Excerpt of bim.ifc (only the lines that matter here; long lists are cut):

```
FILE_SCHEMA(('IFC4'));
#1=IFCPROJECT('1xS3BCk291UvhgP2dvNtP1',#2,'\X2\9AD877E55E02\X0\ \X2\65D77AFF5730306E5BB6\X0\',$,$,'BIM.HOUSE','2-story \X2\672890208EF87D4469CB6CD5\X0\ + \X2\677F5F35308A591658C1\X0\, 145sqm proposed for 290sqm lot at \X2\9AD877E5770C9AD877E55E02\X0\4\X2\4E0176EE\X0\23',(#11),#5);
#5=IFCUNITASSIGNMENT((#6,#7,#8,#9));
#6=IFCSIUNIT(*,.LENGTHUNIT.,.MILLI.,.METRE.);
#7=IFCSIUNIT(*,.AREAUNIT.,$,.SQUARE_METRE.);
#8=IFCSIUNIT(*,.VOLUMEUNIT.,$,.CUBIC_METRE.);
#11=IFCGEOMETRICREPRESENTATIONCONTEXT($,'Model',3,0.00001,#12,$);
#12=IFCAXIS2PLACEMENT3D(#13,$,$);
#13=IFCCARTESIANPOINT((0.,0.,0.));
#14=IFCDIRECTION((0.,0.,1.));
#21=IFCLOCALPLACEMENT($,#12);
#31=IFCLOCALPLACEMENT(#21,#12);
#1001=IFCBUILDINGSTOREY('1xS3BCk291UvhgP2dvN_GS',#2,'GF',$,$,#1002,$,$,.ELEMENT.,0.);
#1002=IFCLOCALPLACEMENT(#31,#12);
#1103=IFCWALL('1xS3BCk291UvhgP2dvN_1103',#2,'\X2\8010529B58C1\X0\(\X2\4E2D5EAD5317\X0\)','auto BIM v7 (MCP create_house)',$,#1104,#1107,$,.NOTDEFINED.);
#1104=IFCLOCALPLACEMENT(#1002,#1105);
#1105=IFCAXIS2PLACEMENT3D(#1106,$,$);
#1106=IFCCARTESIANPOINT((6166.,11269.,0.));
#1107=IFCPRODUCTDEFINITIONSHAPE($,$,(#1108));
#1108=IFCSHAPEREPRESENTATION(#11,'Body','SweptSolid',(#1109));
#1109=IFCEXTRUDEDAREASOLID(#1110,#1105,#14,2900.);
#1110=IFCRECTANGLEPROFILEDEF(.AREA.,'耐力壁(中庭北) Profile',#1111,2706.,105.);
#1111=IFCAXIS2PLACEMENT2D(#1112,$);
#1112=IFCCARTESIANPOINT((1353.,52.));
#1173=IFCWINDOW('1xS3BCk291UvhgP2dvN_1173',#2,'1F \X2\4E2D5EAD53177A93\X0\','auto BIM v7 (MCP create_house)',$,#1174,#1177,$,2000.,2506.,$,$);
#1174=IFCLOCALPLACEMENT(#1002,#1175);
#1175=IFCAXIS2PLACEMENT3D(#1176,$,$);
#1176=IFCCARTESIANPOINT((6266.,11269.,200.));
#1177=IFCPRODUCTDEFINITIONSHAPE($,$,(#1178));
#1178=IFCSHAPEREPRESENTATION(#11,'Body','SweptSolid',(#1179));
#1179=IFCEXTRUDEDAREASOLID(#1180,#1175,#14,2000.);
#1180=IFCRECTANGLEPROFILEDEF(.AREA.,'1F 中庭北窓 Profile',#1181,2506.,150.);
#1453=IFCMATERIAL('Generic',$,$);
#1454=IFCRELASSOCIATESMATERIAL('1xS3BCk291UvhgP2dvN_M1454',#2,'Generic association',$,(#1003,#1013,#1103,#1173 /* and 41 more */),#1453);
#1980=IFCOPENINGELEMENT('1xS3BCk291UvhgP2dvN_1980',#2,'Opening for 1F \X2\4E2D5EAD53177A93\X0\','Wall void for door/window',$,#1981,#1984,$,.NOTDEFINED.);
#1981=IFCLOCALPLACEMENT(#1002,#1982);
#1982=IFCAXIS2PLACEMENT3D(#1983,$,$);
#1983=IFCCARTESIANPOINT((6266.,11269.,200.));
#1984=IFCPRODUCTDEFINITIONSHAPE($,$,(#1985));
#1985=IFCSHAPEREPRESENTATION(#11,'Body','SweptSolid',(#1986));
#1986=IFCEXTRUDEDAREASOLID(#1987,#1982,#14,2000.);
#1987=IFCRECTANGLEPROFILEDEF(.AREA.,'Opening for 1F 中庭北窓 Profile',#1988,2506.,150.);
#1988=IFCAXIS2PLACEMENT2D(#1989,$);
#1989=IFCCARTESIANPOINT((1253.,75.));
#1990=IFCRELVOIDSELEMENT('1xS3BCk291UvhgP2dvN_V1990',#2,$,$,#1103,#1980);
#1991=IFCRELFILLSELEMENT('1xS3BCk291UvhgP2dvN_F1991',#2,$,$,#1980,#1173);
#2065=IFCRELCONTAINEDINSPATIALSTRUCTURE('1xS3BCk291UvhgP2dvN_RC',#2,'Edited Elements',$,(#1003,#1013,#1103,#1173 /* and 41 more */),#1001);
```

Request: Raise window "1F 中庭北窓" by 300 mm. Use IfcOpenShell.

```python
import numpy as np
import ifcopenshell
import ifcopenshell.api.geometry
import ifcopenshell.util.placement
import ifcopenshell.util.unit

model = ifcopenshell.open("bim.ifc")
unit_scale = ifcopenshell.util.unit.calculate_unit_scale(model)

window = model.by_guid("1xS3BCk291UvhgP2dvN_1173")
opening = window.FillsVoids[0].RelatingOpeningElement
dz = 300.0

shift = np.array([0.0, 0.0, dz])
# The window is not placed relative to its opening, so move both.
for product in (opening, window):
    matrix = ifcopenshell.util.placement.get_local_placement(product.ObjectPlacement)
    matrix[:3, 3] += shift
    ifcopenshell.api.geometry.edit_object_placement(model, product=product, matrix=matrix, is_si=False)

print(f"moved by {dz * unit_scale:+.3f} m")

model.write("bim_updated.ifc")
```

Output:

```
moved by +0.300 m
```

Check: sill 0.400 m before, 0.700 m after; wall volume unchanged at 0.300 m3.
